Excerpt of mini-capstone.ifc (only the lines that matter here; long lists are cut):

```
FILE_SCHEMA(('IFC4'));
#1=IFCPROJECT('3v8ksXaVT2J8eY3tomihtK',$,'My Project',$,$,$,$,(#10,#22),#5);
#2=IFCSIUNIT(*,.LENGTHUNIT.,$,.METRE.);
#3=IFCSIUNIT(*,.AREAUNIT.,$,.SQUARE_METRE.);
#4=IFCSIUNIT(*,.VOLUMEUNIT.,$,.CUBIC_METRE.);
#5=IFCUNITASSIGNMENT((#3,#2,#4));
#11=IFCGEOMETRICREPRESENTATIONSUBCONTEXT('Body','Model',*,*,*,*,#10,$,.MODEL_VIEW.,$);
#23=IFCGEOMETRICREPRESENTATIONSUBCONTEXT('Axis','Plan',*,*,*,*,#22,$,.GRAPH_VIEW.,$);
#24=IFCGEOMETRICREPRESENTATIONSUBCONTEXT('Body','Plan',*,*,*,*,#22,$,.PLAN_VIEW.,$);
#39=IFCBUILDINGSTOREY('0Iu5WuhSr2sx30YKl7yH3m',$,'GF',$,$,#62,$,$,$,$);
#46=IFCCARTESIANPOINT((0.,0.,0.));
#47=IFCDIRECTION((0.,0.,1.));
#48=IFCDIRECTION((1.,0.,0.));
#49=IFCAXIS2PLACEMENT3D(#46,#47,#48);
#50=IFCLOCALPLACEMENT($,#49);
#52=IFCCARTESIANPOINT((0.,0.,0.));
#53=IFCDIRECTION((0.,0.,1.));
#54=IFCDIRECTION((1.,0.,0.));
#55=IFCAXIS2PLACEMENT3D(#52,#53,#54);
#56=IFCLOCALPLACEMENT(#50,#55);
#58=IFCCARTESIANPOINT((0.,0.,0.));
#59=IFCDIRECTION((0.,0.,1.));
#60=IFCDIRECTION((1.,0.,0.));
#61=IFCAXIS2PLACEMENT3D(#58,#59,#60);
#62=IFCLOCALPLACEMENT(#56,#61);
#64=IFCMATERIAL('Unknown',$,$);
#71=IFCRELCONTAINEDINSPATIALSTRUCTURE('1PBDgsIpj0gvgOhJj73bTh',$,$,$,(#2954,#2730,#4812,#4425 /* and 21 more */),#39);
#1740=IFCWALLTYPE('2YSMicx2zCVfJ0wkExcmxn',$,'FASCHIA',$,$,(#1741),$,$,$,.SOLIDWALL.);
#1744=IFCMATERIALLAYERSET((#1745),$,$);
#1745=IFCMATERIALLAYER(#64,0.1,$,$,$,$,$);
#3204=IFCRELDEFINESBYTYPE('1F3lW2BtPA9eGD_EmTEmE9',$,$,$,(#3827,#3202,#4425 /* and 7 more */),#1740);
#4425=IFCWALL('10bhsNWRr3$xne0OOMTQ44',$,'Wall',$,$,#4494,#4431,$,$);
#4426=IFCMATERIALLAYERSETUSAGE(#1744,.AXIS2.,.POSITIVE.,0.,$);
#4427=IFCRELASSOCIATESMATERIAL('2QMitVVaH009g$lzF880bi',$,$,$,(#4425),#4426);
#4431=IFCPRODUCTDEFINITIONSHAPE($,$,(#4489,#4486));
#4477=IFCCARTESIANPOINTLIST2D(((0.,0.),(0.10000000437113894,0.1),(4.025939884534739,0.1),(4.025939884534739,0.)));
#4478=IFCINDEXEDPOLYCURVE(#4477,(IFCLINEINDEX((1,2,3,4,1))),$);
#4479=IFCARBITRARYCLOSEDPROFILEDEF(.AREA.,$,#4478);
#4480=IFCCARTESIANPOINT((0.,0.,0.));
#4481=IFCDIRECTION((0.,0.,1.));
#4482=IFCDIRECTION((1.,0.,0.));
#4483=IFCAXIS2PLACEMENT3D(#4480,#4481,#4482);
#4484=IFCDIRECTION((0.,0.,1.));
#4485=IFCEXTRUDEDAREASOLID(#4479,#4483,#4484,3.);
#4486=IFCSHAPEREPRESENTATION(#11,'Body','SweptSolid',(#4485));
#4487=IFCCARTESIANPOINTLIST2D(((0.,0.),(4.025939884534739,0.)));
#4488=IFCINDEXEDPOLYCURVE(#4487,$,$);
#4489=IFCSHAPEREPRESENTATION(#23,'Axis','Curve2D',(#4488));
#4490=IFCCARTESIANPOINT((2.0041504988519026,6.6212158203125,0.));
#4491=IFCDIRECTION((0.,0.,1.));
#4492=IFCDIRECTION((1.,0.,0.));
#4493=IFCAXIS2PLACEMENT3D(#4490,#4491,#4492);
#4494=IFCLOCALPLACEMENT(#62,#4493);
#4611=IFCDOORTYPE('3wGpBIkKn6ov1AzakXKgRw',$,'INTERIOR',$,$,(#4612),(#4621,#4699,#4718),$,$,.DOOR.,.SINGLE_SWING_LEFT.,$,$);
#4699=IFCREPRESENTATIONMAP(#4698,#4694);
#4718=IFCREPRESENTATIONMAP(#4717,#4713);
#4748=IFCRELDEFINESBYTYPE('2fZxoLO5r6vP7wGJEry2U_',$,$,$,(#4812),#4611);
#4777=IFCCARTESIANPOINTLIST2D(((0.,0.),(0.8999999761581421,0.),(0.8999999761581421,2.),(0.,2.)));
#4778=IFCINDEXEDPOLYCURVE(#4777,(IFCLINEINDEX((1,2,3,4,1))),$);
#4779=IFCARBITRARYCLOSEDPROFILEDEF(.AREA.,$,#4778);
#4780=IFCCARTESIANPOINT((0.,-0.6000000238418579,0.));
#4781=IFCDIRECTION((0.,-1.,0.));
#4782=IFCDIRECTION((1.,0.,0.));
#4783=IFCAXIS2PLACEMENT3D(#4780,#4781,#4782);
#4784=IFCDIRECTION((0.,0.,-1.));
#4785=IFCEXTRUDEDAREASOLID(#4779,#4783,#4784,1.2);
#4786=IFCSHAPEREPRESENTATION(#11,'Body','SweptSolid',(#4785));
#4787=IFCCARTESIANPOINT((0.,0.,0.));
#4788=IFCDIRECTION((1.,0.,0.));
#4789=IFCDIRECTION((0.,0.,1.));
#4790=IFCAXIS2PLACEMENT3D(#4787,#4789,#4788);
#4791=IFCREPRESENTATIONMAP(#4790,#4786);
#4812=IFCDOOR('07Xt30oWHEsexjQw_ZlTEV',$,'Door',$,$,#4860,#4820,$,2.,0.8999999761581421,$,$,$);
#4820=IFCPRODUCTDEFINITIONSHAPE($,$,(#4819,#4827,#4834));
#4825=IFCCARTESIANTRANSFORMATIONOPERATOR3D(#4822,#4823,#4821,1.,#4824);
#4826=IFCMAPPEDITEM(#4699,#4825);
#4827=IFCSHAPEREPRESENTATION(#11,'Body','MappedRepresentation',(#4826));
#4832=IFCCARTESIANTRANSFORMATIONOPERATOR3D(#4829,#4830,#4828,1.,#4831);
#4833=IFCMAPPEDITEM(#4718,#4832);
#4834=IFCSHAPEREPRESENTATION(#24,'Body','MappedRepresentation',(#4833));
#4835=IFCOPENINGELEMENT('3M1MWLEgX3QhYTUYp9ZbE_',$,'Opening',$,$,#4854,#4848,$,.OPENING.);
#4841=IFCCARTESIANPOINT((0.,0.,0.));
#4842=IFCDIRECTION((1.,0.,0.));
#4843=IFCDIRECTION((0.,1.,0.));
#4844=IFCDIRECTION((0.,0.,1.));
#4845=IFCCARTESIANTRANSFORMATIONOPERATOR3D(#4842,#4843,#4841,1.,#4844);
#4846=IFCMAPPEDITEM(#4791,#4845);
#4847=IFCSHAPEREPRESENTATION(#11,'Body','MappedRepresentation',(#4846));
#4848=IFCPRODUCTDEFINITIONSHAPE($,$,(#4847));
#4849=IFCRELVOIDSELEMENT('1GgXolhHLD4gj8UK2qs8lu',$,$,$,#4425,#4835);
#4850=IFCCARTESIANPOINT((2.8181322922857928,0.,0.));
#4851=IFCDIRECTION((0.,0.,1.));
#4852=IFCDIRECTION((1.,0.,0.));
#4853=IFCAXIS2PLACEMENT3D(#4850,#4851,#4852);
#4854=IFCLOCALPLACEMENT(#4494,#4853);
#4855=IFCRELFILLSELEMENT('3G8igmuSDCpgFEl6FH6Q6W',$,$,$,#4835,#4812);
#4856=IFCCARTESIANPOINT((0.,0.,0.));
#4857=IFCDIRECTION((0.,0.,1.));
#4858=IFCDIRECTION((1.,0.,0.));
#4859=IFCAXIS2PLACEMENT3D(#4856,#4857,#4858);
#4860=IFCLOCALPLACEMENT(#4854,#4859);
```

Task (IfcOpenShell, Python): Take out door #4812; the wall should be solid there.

```python
import ifcopenshell
import ifcopenshell.api.feature
import ifcopenshell.api.root
import ifcopenshell.geom
import ifcopenshell.util.shape

model = ifcopenshell.open("mini-capstone.ifc")
settings = ifcopenshell.geom.settings()


def volume(element):
    """Net volume in cubic metres, openings subtracted."""
    shape = ifcopenshell.geom.create_shape(settings, element)
    return ifcopenshell.util.shape.get_volume(shape.geometry)


door = model.by_id(4812)
opening = door.FillsVoids[0].RelatingOpeningElement
wall = opening.VoidsElements[0].RelatingBuildingElement
before = volume(wall)

ifcopenshell.api.root.remove_product(model, product=door)
ifcopenshell.api.feature.remove_feature(model, feature=opening)

after = volume(wall)

print(f"wall volume {before:.3f} -> {after:.3f} m3")

model.write("mini-capstone-out.ifc")
```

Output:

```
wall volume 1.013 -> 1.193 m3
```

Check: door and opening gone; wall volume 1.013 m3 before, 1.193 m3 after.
